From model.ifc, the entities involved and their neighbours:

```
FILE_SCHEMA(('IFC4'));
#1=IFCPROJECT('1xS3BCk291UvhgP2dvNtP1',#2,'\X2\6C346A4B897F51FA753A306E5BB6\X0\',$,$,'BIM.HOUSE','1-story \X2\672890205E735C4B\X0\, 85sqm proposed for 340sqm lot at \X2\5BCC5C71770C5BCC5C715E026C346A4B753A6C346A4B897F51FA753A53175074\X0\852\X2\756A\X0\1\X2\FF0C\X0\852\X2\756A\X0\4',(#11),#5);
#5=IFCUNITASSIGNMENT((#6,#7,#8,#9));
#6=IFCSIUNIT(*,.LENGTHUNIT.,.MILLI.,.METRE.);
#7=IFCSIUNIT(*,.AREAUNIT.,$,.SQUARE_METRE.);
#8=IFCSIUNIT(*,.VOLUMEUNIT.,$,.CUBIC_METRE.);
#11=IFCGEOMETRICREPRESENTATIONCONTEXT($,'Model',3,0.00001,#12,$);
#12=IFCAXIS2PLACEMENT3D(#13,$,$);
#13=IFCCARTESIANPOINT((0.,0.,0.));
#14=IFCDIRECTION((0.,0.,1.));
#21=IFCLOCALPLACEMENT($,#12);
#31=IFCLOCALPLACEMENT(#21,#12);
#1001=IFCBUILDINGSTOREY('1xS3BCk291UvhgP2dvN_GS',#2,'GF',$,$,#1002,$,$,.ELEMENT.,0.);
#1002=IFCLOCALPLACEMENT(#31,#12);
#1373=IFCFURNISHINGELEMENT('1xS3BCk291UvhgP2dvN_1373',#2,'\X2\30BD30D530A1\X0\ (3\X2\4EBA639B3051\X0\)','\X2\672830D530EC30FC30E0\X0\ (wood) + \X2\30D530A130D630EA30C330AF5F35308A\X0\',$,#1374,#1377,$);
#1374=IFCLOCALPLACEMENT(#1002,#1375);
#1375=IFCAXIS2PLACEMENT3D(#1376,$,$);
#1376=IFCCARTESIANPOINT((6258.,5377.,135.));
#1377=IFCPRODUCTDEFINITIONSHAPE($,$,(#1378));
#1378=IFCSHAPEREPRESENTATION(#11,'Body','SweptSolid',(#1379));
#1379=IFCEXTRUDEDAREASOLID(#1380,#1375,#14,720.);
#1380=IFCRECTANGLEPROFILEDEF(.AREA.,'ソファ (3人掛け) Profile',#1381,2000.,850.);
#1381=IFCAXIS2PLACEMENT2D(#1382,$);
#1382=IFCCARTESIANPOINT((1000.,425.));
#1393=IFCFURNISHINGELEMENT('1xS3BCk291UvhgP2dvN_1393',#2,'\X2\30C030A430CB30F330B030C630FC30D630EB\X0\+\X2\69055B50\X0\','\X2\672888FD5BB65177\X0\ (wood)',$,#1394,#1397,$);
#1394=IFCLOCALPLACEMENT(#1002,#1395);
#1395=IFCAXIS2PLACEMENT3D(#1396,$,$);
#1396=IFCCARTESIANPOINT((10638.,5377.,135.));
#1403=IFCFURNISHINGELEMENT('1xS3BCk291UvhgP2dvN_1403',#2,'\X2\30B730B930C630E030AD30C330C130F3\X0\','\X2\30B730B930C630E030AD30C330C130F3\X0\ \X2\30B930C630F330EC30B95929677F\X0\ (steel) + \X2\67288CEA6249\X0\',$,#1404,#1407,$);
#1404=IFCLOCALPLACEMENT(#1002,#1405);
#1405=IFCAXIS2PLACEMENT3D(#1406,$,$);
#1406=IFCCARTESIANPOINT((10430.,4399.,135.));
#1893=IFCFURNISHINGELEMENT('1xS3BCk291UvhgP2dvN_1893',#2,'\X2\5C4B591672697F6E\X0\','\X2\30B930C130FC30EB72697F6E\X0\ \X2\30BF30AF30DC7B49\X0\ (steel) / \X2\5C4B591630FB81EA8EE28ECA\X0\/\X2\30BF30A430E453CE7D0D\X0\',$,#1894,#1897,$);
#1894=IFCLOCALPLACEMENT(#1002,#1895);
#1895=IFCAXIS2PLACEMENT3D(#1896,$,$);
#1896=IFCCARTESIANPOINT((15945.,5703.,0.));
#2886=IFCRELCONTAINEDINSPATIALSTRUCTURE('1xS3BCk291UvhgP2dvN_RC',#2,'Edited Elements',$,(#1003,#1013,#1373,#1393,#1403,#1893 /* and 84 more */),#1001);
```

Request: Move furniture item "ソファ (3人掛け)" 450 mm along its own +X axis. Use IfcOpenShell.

```python
import ifcopenshell
import ifcopenshell.api.geometry
import ifcopenshell.util.placement

model = ifcopenshell.open("model.ifc")

item = model.by_guid("1xS3BCk291UvhgP2dvN_1373")
matrix = ifcopenshell.util.placement.get_local_placement(item.ObjectPlacement)
matrix[:3, 3] += matrix[:3, 0] * 450.0
ifcopenshell.api.geometry.edit_object_placement(model, product=item, matrix=matrix, is_si=False)

print(ifcopenshell.util.placement.get_local_placement(item.ObjectPlacement).round(3) + 0.0)

model.write("model_v2.ifc")
```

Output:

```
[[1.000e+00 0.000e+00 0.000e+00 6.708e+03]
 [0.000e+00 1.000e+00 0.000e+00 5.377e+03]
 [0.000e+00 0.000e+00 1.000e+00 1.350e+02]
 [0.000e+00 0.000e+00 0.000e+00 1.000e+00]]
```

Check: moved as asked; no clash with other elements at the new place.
